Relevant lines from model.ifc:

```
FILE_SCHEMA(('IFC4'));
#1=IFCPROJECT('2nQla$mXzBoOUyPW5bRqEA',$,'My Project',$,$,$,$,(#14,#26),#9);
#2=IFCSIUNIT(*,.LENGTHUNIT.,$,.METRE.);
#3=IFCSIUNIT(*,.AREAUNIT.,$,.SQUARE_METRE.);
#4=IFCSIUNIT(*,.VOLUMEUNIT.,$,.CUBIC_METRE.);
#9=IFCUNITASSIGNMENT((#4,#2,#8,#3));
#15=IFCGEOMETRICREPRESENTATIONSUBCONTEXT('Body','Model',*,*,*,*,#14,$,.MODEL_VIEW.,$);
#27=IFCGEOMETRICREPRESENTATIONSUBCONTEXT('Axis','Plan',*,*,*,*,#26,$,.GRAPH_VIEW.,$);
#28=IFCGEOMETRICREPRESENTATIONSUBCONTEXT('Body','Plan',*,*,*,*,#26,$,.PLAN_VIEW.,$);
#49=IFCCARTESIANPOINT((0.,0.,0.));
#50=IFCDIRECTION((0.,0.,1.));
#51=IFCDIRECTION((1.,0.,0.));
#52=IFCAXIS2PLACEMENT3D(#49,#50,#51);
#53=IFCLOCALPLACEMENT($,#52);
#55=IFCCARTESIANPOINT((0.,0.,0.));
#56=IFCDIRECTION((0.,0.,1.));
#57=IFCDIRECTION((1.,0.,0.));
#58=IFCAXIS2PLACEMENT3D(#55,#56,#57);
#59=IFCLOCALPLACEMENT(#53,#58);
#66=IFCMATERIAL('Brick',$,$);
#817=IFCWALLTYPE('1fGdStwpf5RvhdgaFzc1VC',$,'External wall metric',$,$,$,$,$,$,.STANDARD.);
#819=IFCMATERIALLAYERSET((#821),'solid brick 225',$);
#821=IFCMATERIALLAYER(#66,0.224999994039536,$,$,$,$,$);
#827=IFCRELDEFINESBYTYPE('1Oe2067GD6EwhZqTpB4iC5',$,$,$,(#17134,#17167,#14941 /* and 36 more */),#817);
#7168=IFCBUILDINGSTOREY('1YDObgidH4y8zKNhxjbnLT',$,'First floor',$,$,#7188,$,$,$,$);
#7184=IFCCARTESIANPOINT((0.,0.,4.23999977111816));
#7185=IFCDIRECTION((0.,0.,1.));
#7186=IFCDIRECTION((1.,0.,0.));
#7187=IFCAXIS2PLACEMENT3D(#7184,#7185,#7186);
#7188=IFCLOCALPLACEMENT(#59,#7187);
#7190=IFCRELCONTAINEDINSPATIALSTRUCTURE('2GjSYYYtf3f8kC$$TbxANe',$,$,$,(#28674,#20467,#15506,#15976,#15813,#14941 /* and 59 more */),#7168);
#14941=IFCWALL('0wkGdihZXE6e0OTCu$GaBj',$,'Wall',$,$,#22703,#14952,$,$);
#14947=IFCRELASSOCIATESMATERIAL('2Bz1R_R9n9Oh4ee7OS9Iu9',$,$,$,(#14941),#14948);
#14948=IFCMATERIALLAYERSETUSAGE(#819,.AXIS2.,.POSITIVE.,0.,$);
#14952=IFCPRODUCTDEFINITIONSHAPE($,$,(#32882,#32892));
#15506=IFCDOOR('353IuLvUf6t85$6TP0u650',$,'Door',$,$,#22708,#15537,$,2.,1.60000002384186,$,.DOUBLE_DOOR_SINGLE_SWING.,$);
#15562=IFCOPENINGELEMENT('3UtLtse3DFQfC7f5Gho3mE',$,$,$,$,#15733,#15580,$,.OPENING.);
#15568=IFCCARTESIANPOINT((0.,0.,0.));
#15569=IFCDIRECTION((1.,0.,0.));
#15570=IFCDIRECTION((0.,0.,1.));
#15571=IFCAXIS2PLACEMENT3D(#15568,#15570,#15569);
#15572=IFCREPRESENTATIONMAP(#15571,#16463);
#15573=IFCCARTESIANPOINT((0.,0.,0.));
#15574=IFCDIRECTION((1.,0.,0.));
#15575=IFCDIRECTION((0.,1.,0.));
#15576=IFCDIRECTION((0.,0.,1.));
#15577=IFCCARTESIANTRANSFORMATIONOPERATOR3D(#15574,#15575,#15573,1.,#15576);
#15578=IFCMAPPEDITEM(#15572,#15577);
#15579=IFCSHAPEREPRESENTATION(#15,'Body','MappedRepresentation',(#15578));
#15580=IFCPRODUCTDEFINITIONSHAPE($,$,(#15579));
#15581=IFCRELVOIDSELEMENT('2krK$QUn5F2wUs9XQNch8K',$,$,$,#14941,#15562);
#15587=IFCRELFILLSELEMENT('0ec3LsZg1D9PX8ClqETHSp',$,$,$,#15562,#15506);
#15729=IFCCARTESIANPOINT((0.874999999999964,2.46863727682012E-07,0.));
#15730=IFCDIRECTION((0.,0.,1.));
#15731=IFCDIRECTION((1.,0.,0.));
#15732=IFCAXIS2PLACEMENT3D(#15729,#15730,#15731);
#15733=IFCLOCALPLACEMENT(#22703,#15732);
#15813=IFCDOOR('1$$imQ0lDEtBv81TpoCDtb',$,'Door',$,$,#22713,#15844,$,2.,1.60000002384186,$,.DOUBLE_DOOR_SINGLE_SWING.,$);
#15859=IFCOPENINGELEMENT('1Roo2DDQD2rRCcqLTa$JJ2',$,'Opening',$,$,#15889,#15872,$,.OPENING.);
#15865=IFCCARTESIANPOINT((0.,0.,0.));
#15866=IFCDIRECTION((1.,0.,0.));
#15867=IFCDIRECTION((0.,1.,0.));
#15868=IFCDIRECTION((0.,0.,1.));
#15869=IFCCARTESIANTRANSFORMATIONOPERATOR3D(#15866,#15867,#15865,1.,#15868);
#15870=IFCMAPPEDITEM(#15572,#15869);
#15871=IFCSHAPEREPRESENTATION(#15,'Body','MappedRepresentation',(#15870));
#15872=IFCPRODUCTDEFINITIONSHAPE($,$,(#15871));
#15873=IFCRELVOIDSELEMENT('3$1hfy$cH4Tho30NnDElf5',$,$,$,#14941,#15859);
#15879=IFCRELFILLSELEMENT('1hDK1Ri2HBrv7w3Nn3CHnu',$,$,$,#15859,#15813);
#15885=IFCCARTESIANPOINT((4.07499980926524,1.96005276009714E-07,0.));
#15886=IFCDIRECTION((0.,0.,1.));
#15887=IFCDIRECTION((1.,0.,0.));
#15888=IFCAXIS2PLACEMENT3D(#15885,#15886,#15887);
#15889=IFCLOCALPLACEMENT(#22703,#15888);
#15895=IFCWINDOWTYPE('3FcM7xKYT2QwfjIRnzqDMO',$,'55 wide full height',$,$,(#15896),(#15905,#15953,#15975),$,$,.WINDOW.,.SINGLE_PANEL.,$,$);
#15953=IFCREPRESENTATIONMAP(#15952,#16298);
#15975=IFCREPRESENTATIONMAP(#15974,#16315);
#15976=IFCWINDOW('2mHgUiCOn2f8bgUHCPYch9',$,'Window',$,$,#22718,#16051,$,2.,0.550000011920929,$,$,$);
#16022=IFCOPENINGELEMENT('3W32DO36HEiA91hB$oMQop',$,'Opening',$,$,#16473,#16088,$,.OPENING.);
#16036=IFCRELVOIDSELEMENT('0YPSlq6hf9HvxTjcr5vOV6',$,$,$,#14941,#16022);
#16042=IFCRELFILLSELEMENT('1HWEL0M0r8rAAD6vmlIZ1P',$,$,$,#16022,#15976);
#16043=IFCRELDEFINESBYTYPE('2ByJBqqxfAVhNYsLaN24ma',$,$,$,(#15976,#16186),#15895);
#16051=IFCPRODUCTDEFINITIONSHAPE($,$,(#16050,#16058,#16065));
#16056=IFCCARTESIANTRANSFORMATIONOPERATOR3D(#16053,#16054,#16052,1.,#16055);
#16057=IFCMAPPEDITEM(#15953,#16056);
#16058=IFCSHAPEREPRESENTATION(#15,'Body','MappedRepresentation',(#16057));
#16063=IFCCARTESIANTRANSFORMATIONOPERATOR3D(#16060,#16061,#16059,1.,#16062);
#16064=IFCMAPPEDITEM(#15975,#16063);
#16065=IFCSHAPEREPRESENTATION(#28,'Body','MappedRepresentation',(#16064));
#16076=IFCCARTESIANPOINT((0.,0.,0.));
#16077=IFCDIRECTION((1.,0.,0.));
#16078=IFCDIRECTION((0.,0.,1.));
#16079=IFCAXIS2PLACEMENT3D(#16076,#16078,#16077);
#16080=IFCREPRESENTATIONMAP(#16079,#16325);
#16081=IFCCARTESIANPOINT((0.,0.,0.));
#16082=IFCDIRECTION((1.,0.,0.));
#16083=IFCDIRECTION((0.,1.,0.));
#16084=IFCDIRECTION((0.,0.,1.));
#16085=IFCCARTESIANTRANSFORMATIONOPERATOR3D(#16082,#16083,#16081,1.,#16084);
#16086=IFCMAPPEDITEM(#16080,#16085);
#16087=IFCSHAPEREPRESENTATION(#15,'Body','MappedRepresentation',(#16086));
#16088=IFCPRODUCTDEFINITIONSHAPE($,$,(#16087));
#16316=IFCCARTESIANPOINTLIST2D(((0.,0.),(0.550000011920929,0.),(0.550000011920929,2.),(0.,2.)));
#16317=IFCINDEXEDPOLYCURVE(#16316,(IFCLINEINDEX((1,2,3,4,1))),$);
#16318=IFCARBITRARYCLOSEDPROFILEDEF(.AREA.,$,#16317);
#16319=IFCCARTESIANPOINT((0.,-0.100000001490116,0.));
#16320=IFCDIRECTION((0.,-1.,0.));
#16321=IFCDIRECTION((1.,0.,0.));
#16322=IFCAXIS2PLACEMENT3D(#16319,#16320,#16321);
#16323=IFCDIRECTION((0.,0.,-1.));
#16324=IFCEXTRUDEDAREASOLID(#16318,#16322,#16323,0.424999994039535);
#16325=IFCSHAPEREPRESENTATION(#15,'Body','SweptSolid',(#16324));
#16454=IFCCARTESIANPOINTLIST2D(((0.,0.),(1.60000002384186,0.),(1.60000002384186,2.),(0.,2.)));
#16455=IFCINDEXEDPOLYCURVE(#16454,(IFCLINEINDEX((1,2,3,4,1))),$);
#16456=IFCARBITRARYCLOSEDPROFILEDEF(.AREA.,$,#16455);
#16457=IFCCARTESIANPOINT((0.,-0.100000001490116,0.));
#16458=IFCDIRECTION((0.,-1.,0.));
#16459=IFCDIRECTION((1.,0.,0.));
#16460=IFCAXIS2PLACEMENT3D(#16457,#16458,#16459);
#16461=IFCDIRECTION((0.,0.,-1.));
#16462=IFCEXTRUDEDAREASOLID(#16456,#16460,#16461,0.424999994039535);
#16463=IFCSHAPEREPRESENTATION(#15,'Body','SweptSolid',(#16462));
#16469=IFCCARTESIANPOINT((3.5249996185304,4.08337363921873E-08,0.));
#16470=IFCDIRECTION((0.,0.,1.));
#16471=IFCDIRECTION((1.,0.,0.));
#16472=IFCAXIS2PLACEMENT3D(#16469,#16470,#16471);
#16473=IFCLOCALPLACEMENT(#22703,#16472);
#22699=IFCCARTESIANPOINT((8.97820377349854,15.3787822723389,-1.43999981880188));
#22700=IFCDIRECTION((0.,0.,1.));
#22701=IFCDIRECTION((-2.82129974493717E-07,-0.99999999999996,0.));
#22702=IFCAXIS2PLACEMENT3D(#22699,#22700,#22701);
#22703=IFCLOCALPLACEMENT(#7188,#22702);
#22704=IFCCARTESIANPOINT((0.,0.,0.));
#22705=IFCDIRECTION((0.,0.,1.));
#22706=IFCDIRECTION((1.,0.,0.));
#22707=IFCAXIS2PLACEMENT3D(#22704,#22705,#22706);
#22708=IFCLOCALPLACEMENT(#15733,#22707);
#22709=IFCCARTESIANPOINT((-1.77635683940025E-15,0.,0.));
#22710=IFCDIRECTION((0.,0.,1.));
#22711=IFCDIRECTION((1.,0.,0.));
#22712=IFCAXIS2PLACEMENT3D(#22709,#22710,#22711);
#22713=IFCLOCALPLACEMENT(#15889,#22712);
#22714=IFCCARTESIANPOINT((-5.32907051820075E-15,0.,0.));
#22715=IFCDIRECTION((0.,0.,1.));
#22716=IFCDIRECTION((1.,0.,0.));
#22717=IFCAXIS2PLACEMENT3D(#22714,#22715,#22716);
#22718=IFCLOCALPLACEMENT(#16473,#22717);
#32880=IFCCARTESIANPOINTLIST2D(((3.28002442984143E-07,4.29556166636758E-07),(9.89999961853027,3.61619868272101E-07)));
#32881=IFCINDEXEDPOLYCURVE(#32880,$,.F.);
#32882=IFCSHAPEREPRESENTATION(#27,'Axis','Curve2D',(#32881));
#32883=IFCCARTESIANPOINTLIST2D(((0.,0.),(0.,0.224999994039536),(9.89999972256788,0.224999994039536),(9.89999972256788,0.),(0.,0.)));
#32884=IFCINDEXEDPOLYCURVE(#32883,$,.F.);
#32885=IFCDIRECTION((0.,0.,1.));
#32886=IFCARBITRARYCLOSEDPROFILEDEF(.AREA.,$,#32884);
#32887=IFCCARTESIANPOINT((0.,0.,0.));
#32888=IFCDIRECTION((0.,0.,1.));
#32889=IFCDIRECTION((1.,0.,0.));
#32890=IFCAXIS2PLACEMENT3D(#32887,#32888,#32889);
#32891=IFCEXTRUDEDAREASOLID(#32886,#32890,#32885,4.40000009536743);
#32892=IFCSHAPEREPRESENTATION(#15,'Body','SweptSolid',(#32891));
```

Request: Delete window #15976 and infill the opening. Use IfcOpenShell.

```python
import ifcopenshell
import ifcopenshell.api.feature
import ifcopenshell.api.root
import ifcopenshell.geom
import ifcopenshell.util.shape

model = ifcopenshell.open("model.ifc")
settings = ifcopenshell.geom.settings()


def volume(element):
    """Net volume in cubic metres, openings subtracted."""
    shape = ifcopenshell.geom.create_shape(settings, element)
    return ifcopenshell.util.shape.get_volume(shape.geometry)


window = model.by_guid("2mHgUiCOn2f8bgUHCPYch9")
opening = window.FillsVoids[0].RelatingOpeningElement
wall = opening.VoidsElements[0].RelatingBuildingElement
before = volume(wall)

ifcopenshell.api.root.remove_product(model, product=window)
ifcopenshell.api.feature.remove_feature(model, feature=opening)

after = volume(wall)

print(f"wall volume {before:.3f} -> {after:.3f} m3")

model.write("model-out.ifc")
```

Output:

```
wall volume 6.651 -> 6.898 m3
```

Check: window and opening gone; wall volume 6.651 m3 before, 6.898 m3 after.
